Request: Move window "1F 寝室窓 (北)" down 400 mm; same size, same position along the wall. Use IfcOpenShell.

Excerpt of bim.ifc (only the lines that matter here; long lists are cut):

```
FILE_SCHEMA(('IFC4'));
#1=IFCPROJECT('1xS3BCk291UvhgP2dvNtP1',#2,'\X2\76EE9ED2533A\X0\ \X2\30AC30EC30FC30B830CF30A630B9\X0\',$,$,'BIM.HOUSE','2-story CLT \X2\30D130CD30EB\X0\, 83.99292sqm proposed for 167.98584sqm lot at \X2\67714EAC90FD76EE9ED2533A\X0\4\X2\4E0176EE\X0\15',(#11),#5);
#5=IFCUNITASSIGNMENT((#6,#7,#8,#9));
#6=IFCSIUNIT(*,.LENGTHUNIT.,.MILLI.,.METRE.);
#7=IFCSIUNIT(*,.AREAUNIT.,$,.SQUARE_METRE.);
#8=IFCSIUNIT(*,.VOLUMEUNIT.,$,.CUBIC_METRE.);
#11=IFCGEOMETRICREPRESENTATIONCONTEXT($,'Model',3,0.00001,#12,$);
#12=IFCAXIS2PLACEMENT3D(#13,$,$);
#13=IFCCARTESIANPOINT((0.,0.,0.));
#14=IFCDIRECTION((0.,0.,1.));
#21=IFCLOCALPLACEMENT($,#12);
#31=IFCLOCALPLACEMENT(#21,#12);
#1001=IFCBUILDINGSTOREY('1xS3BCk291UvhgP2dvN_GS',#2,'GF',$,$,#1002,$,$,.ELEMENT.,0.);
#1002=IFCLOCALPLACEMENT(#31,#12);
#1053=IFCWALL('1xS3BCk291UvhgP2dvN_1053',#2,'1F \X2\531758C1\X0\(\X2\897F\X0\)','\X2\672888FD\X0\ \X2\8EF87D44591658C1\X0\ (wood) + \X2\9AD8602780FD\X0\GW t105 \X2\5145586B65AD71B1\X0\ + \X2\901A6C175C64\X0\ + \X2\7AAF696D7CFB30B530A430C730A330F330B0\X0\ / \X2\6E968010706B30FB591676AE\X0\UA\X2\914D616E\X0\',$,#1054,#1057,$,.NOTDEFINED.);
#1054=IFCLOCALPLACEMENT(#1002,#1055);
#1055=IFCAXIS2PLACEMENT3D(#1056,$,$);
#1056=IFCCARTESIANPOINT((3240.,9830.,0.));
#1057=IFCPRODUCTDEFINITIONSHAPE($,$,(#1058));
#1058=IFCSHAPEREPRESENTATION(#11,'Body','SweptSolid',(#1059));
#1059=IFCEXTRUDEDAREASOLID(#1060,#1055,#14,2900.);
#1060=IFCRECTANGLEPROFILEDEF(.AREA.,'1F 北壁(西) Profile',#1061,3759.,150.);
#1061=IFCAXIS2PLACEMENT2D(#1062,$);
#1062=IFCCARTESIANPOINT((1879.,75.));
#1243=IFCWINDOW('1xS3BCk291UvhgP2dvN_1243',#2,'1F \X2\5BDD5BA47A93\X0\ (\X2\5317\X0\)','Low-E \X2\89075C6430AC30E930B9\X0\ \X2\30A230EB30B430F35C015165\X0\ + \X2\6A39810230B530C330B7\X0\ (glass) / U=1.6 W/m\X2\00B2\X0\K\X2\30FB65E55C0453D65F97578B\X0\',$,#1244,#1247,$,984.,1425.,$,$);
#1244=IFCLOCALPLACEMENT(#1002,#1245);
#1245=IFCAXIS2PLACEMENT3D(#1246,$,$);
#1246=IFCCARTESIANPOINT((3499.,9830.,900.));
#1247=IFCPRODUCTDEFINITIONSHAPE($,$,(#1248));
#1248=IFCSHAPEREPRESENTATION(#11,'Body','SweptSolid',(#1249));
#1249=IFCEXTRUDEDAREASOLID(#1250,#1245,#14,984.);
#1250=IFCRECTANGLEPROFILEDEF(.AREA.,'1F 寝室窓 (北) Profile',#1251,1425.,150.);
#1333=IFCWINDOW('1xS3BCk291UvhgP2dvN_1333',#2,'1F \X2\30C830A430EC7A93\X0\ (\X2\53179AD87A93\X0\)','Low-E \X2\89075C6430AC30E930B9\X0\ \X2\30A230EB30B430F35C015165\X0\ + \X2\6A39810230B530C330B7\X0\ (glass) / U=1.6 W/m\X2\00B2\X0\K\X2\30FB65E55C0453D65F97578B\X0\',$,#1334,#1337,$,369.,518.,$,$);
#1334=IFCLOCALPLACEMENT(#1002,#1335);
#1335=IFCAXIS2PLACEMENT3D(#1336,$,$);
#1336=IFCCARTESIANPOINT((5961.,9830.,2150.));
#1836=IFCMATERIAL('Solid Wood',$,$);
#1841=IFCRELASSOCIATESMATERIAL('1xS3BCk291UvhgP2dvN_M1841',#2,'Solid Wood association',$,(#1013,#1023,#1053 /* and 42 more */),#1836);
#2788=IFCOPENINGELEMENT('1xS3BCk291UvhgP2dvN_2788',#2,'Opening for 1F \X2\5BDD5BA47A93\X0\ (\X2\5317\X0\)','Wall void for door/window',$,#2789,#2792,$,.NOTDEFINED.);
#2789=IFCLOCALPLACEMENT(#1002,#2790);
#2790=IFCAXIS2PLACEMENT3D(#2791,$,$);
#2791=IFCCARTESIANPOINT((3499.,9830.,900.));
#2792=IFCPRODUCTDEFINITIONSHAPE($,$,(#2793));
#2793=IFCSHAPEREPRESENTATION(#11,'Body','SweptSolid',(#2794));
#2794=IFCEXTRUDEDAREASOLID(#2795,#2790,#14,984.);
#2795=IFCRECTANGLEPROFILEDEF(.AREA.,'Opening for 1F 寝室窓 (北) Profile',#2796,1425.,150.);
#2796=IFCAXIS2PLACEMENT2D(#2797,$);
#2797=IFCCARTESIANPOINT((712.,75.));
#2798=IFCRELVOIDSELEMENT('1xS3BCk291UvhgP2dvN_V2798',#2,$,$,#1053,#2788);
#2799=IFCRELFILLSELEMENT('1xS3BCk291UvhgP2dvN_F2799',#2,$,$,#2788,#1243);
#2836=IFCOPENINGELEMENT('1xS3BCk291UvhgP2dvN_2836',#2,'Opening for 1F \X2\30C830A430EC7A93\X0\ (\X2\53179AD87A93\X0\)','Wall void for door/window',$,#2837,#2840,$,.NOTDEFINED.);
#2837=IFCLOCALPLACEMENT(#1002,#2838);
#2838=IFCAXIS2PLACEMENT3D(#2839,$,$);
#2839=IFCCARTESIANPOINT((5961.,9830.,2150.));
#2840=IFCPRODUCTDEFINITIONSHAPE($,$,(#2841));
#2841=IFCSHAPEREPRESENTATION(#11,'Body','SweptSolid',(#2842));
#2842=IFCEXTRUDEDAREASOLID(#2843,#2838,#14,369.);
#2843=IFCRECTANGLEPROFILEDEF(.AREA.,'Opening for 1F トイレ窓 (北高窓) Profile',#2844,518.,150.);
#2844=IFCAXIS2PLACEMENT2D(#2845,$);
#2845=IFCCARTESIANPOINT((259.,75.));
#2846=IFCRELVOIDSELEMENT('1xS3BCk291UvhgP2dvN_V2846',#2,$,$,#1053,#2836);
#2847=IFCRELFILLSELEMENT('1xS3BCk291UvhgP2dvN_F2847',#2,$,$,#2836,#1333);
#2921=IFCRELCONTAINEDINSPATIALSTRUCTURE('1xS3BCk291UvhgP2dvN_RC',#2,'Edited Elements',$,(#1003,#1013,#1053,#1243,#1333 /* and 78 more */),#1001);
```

```python
import numpy as np
import ifcopenshell
import ifcopenshell.api.geometry
import ifcopenshell.util.placement
import ifcopenshell.util.unit

model = ifcopenshell.open("bim.ifc")
unit_scale = ifcopenshell.util.unit.calculate_unit_scale(model)

window = model.by_id(1243)
opening = window.FillsVoids[0].RelatingOpeningElement
dz = -400.0

shift = np.array([0.0, 0.0, dz])
# The window is not placed relative to its opening, so move both.
for product in (opening, window):
    matrix = ifcopenshell.util.placement.get_local_placement(product.ObjectPlacement)
    matrix[:3, 3] += shift
    ifcopenshell.api.geometry.edit_object_placement(model, product=product, matrix=matrix, is_si=False)

print(f"moved by {dz * unit_scale:+.3f} m")

model.write("bim-out.ifc")
```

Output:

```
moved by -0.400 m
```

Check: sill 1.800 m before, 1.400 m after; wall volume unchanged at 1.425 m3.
